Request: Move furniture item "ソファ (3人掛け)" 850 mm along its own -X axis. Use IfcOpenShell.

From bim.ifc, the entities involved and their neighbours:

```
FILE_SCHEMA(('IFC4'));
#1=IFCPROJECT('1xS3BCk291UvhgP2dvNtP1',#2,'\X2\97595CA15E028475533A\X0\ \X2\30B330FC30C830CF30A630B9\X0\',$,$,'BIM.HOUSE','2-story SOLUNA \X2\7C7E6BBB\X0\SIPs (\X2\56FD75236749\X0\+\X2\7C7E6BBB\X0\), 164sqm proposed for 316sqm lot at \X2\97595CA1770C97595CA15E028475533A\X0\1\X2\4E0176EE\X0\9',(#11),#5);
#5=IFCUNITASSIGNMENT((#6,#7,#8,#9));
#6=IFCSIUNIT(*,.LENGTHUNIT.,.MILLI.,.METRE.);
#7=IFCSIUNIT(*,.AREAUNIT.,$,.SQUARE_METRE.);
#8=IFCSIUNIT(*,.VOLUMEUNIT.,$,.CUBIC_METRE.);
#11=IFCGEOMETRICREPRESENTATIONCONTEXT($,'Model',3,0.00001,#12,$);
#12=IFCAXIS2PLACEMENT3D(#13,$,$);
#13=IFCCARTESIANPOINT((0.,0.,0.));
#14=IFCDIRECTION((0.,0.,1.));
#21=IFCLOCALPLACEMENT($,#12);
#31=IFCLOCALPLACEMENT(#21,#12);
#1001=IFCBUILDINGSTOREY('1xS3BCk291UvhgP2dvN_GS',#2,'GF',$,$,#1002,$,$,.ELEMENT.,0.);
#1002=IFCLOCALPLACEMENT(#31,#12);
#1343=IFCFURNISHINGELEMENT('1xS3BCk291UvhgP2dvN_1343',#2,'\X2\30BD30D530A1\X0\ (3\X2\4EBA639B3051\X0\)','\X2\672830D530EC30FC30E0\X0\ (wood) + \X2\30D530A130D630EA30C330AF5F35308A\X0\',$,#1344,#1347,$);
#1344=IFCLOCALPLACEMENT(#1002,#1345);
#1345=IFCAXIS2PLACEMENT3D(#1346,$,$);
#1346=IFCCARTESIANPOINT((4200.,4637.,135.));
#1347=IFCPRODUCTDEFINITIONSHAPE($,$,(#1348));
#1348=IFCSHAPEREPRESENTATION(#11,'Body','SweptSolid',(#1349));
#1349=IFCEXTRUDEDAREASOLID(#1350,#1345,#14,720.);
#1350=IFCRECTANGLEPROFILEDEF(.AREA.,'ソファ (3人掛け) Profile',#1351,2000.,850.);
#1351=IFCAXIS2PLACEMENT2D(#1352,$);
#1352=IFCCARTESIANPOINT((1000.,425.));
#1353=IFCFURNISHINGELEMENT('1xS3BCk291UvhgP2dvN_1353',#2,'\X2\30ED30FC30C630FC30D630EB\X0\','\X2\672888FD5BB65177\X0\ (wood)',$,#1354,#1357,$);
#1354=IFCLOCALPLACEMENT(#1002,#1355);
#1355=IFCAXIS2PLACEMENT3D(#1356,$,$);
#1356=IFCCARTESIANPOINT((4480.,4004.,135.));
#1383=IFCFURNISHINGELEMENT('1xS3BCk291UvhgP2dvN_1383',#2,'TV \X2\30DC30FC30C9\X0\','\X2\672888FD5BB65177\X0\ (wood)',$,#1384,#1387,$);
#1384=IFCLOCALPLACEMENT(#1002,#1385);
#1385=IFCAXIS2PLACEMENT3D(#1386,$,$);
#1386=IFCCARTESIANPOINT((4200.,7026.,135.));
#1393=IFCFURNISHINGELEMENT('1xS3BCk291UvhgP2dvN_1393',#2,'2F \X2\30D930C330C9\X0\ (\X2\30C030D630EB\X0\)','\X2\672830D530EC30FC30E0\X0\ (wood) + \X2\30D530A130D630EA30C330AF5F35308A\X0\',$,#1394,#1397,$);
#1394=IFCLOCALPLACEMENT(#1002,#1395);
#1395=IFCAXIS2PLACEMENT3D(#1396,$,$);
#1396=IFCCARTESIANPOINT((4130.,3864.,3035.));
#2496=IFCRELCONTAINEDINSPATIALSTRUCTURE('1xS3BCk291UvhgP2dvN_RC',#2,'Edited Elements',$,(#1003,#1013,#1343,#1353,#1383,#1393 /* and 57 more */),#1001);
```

```python
import ifcopenshell
import ifcopenshell.api.geometry
import ifcopenshell.util.placement
import ifcopenshell.util.unit

model = ifcopenshell.open("bim.ifc")
unit_scale = ifcopenshell.util.unit.calculate_unit_scale(model)

item = model.by_guid("1xS3BCk291UvhgP2dvN_1343")
matrix = ifcopenshell.util.placement.get_local_placement(item.ObjectPlacement)
matrix[:3, 3] -= matrix[:3, 0] * 0.85 / unit_scale
ifcopenshell.api.geometry.edit_object_placement(model, product=item, matrix=matrix, is_si=False)

print(ifcopenshell.util.placement.get_local_placement(item.ObjectPlacement).round(3) + 0.0)

model.write("bim_rev.ifc")
```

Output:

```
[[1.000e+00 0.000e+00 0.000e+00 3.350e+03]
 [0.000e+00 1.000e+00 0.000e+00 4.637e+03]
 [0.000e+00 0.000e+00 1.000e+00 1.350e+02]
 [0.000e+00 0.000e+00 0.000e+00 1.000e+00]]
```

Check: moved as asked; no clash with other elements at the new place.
